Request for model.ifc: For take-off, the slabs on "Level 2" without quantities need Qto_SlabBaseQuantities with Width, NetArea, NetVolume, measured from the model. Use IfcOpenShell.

First a look at what the model holds.

```python
import ifcopenshell
import ifcopenshell.util.element
import ifcopenshell.util.unit

model = ifcopenshell.open("model.ifc")
print(model.schema)
for unit_type in ("LENGTHUNIT", "AREAUNIT", "VOLUMEUNIT"):
    print(unit_type, ifcopenshell.util.unit.calculate_unit_scale(model, unit_type))
storey = next(s for s in model.by_type("IfcBuildingStorey") if s.Name == "Level 2")
slabs = [e for e in ifcopenshell.util.element.get_decomposition(storey) if e.is_a("IfcSlab")]
for e in sorted(slabs, key=lambda e: e.id()):
    print(e.id(), e.is_a(), e.Name, list(ifcopenshell.util.element.get_psets(e, qtos_only=True)), sep=" | ")
```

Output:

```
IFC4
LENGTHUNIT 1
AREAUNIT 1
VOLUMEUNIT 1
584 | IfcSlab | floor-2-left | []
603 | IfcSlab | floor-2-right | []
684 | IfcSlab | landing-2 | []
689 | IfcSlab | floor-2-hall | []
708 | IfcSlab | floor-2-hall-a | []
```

```python
import ifcopenshell
import ifcopenshell.api.pset
import ifcopenshell.geom
import ifcopenshell.util.element
import ifcopenshell.util.shape
import ifcopenshell.util.unit

model = ifcopenshell.open("model.ifc")
unit_scale = ifcopenshell.util.unit.calculate_unit_scale(model)
area_scale = ifcopenshell.util.unit.calculate_unit_scale(model, "AREAUNIT")
volume_scale = ifcopenshell.util.unit.calculate_unit_scale(model, "VOLUMEUNIT")
settings = ifcopenshell.geom.settings()

storey = next(s for s in model.by_type("IfcBuildingStorey") if s.Name == "Level 2")
slabs = [e for e in ifcopenshell.util.element.get_decomposition(storey) if e.is_a("IfcSlab")]

for e in sorted(slabs, key=lambda e: e.id()):
    if ifcopenshell.util.element.get_psets(e, qtos_only=True, should_inherit=False):
        continue
    # Geometry comes back in metres, in the element's own axes.
    shape = ifcopenshell.geom.create_shape(settings, e)
    values = {
        "Width": ifcopenshell.util.shape.get_z(shape.geometry) / unit_scale,
        "NetArea": ifcopenshell.util.shape.get_footprint_area(shape.geometry) / area_scale,
        "NetVolume": ifcopenshell.util.shape.get_volume(shape.geometry) / volume_scale,
    }
    qto = ifcopenshell.api.pset.add_qto(model, product=e, name="Qto_SlabBaseQuantities")
    ifcopenshell.api.pset.edit_qto(model, qto=qto, properties=values)
    print(e.id(), {k: round(v, 3) for k, v in values.items()})

model.write("model_edited.ifc")
```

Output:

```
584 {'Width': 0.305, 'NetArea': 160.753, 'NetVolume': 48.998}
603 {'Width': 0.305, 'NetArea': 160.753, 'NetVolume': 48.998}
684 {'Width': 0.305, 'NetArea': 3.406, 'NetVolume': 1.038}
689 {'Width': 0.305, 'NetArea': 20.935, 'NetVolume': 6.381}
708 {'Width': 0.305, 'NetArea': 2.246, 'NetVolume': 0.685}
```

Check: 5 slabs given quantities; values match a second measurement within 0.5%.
